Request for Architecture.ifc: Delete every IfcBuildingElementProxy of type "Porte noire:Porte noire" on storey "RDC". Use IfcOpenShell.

First a look at what the model holds.

```python
import ifcopenshell
import ifcopenshell.util.element

model = ifcopenshell.open("Architecture.ifc")
print(model.schema)
storey = next(s for s in model.by_type("IfcBuildingStorey") if s.Name == "RDC")
proxies = [e for e in ifcopenshell.util.element.get_decomposition(storey) if e.is_a("IfcBuildingElementProxy")]
seen = {}
for e in proxies:
    element_type = ifcopenshell.util.element.get_type(e)
    name = element_type.Name if element_type not in (None, e) else None
    seen[name] = seen.get(name, 0) + 1
for name, count in sorted(seen.items(), key=str):
    print(count, "x", name)
```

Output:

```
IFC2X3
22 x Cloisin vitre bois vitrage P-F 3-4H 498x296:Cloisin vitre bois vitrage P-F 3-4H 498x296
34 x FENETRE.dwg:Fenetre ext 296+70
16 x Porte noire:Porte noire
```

```python
import ifcopenshell
import ifcopenshell.api.root
import ifcopenshell.util.element

model = ifcopenshell.open("Architecture.ifc")

storey = next(s for s in model.by_type("IfcBuildingStorey") if s.Name == "RDC")
proxies = [e for e in ifcopenshell.util.element.get_decomposition(storey) if e.is_a("IfcBuildingElementProxy")]
targets = [e for e in proxies if (t := ifcopenshell.util.element.get_type(e)) not in (None, e) and t.Name == "Porte noire:Porte noire"]

for e in targets:
    ifcopenshell.api.root.remove_product(model, product=e)
print(len(targets), "removed")

model.write("Architecture_rev.ifc")
```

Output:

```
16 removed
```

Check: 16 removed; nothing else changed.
